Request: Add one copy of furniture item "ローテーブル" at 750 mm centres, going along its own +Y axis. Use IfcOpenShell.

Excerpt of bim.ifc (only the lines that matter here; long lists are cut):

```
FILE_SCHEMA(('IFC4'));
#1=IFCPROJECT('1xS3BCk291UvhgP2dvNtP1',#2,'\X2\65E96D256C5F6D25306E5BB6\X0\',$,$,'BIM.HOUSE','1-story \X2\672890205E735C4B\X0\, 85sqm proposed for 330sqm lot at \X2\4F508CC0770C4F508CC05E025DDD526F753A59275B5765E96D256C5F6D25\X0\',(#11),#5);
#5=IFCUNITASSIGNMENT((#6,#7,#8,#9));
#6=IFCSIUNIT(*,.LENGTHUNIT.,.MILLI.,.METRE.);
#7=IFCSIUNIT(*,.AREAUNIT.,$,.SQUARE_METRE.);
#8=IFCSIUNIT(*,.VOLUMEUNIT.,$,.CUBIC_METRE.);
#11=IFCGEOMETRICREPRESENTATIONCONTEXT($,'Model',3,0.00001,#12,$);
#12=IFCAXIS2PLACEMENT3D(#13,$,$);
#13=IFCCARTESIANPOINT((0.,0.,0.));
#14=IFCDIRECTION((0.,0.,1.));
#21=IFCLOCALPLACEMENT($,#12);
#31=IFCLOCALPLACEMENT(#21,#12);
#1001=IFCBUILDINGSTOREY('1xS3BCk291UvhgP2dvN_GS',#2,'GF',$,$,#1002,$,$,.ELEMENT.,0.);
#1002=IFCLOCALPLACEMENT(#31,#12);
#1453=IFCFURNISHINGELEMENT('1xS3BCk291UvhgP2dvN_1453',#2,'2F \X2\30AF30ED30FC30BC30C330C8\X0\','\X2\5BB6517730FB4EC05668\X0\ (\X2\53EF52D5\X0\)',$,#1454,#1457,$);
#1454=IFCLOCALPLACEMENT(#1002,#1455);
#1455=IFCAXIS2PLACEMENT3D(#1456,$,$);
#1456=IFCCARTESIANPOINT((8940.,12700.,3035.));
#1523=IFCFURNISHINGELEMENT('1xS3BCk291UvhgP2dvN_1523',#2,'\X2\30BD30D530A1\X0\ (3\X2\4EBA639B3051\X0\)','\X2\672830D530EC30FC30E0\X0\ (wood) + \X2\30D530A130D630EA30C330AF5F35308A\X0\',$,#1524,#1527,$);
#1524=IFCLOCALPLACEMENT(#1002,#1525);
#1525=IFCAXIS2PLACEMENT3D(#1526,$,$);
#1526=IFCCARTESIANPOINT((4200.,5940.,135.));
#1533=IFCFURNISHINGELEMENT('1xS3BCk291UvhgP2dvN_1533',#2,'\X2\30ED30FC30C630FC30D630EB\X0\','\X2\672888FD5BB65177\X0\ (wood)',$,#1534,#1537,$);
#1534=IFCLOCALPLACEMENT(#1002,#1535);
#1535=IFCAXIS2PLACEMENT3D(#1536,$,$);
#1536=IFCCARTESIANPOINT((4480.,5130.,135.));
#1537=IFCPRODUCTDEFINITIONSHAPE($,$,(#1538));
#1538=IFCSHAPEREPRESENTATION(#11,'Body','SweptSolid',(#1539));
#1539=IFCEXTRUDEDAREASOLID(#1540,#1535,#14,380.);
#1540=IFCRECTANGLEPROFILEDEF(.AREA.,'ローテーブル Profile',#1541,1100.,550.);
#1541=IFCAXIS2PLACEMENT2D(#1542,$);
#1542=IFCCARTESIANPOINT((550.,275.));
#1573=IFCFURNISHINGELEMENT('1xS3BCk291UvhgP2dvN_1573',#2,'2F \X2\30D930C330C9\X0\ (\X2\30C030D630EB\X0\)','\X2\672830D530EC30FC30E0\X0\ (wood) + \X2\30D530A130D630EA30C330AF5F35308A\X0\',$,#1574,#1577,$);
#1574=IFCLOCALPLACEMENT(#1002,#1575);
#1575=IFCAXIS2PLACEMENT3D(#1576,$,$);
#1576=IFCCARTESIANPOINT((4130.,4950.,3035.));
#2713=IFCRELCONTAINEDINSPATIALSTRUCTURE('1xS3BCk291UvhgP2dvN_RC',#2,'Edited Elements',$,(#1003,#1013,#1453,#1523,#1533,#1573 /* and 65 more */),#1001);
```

```python
import ifcopenshell
import ifcopenshell.api.geometry
import ifcopenshell.api.root
import ifcopenshell.util.element
import ifcopenshell.util.placement

model = ifcopenshell.open("bim.ifc")


def reuse_history(source, copy):
    """copy_class also copies each property set's owner history, people and application; keep the originals."""
    for rel in copy.IsDefinedBy:
        if rel.is_a("IfcRelDefinesByProperties") and (history := rel.RelatingPropertyDefinition.OwnerHistory):
            rel.RelatingPropertyDefinition.OwnerHistory = source.OwnerHistory
            ifcopenshell.util.element.remove_deep2(model, history)


source = model.by_id(1533)
base = ifcopenshell.util.placement.get_local_placement(source.ObjectPlacement)
step = base[:3, 1] * 750.0

for i in range(1, 2):
    copy = ifcopenshell.api.root.copy_class(model, product=source)
    copy.Representation = ifcopenshell.util.element.copy_deep(
        model, source.Representation, exclude=["IfcGeometricRepresentationContext", "IfcRepresentationMap"]
    )
    reuse_history(source, copy)
    matrix = base.copy()
    matrix[:3, 3] += i * step
    print("added at", matrix[:3, 3].round(3) + 0.0)
    ifcopenshell.api.geometry.edit_object_placement(model, product=copy, matrix=matrix, is_si=False)

model.write("bim_edited.ifc")
```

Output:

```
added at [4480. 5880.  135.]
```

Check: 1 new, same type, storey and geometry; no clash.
